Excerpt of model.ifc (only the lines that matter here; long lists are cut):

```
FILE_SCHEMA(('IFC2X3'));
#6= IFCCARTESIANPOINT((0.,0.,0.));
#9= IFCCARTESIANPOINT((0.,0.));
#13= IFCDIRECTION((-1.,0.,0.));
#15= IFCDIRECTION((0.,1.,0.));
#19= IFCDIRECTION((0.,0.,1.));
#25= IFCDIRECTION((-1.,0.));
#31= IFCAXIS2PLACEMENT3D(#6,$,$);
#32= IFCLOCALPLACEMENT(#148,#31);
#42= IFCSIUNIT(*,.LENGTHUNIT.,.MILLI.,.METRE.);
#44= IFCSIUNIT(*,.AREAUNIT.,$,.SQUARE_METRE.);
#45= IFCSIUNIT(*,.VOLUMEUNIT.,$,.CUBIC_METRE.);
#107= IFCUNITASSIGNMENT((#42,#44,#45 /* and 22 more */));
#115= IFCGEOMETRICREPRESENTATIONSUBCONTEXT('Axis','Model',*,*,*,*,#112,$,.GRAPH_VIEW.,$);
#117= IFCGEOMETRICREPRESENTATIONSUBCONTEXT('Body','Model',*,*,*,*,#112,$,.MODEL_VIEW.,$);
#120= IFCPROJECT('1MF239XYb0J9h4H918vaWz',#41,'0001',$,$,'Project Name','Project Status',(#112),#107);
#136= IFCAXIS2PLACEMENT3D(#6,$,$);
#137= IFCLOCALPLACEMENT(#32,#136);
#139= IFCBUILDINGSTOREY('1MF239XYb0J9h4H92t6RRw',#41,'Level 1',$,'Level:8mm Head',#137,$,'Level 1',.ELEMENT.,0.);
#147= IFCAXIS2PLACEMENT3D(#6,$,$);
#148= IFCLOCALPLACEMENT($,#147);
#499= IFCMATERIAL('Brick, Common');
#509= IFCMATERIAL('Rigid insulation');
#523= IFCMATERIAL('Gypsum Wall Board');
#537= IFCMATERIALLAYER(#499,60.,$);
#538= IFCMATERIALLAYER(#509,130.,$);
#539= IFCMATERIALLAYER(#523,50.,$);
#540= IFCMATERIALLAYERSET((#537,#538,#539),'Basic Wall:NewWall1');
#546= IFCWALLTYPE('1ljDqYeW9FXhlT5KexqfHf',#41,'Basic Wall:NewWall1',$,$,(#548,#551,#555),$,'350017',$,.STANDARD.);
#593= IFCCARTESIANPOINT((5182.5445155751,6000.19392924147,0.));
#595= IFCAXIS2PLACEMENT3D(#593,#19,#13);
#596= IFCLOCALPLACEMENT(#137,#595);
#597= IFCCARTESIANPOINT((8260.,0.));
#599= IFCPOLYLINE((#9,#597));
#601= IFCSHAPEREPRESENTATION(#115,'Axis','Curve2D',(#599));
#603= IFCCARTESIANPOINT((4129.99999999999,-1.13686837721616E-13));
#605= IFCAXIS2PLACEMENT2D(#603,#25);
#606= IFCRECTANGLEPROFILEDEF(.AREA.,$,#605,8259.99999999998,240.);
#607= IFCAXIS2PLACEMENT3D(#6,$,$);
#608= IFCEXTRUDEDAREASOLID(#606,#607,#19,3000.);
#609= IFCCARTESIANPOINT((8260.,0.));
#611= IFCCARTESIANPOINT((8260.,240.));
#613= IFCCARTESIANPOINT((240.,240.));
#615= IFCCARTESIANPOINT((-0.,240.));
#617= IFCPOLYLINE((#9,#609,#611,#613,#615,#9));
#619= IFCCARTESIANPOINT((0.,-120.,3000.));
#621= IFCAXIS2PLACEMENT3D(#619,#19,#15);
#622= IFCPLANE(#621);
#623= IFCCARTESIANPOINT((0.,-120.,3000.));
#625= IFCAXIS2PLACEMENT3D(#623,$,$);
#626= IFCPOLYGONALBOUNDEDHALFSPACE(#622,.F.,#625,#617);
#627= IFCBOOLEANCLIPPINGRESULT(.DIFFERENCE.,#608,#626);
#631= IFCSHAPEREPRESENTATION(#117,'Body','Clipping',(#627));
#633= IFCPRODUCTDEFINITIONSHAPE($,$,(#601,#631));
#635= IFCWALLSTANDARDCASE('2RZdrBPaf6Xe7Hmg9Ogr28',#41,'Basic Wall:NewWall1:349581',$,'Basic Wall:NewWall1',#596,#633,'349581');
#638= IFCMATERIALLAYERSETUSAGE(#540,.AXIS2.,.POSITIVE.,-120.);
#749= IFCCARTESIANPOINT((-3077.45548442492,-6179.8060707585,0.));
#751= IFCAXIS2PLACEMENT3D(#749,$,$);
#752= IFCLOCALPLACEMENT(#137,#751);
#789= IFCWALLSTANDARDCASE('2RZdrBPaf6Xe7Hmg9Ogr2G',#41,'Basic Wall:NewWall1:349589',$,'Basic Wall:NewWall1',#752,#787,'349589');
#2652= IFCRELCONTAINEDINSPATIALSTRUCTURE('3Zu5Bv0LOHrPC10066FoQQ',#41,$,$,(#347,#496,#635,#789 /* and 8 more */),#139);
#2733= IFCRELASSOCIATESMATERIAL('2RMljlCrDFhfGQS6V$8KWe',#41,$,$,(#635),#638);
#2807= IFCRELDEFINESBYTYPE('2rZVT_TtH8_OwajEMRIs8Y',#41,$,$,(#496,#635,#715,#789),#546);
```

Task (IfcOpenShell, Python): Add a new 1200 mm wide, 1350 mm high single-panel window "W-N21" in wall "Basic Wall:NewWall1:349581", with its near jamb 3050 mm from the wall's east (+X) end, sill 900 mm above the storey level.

```python
import numpy as np
import ifcopenshell
import ifcopenshell.api.feature
import ifcopenshell.api.geometry
import ifcopenshell.api.root
import ifcopenshell.api.spatial
import ifcopenshell.api.type
import ifcopenshell.geom
import ifcopenshell.util.element
import ifcopenshell.util.placement
import ifcopenshell.util.representation
import ifcopenshell.util.shape
import ifcopenshell.util.unit

model = ifcopenshell.open("model.ifc")
unit_scale = ifcopenshell.util.unit.calculate_unit_scale(model)
settings = ifcopenshell.geom.settings()


def volume(element):
    """Net volume in cubic metres, openings subtracted."""
    shape = ifcopenshell.geom.create_shape(settings, element)
    return ifcopenshell.util.shape.get_volume(shape.geometry)


wall = model.by_guid("2RZdrBPaf6Xe7Hmg9Ogr28")
storey = ifcopenshell.util.element.get_container(wall, ifc_class="IfcBuildingStorey")
context = ifcopenshell.util.representation.get_context(model, "Model", "Body", "MODEL_VIEW")
before = volume(wall)

width, height, from_end, sill = 1.2, 1.35, 3.05, 0.9  # metres

# The wall runs along its own X axis, and the end named is its -X end.
wall_shape = ifcopenshell.geom.create_shape(settings, wall)
x, y, z = ifcopenshell.util.shape.get_vertices(wall_shape.geometry).T
start = x.min() + from_end
face, thickness = float(y.min()), float(y.max() - y.min())
wall_matrix = ifcopenshell.util.placement.get_local_placement(wall.ObjectPlacement)
level = ifcopenshell.util.placement.get_local_placement(storey.ObjectPlacement)[2, 3]


def in_wall(x, y):
    """Placement at x, y metres in the wall's axes, at sill height."""
    matrix = wall_matrix.copy()
    matrix[:, 3] = wall_matrix @ np.array([x / unit_scale, y / unit_scale, 0.0, 1.0])
    matrix[2, 3] = level + sill / unit_scale
    return matrix


# Opening: a box that overshoots both wall faces by 50 mm.
opening = ifcopenshell.api.root.create_entity(model, ifc_class="IfcOpeningElement")
box = ifcopenshell.api.geometry.add_wall_representation(
    model, context=context, length=width, height=height, thickness=thickness + 0.1
)
ifcopenshell.api.geometry.assign_representation(model, product=opening, representation=box)
ifcopenshell.api.geometry.edit_object_placement(model, product=opening, matrix=in_wall(start, face - 0.05), is_si=False)
ifcopenshell.api.feature.add_feature(model, feature=opening, element=wall)

window = ifcopenshell.api.root.create_entity(model, ifc_class="IfcWindow", name="W-N21")
window.OverallWidth, window.OverallHeight = width / unit_scale, height / unit_scale
body = ifcopenshell.api.geometry.add_window_representation(
    model,
    context=context,
    overall_width=window.OverallWidth,
    overall_height=window.OverallHeight,
    partition_type="SINGLE_PANEL",
)
ifcopenshell.api.geometry.assign_representation(model, product=window, representation=body)
ifcopenshell.api.spatial.assign_container(model, products=[window], relating_structure=storey)
fills = ifcopenshell.api.feature.add_filling(model, opening=opening, element=window)
fills.OwnerHistory = window.OwnerHistory  # required in IFC2X3

# IFC2X3 keeps the operation on the window style.
style = ifcopenshell.api.root.create_entity(model, ifc_class="IfcWindowStyle", name="W-N21")
style.OperationType, style.ConstructionType = "SINGLE_PANEL", "NOTDEFINED"
style.ParameterTakesPrecedence = style.Sizeable = False
ifcopenshell.api.type.assign_type(model, related_objects=[window], relating_type=style)

# Centre the window in the wall's thickness.
ifcopenshell.api.geometry.edit_object_placement(model, product=window, matrix=in_wall(start, face), is_si=False)
window_shape = ifcopenshell.geom.create_shape(settings, window)
depth = ifcopenshell.util.shape.get_vertices(window_shape.geometry)[:, 1]
offset = face + thickness / 2 - (depth.min() + depth.max()) / 2
ifcopenshell.api.geometry.edit_object_placement(model, product=window, matrix=in_wall(start, offset), is_si=False)

after = volume(wall)

print(f"wall volume {before:.3f} -> {after:.3f} m3")

model.write("model_edited.ifc")
```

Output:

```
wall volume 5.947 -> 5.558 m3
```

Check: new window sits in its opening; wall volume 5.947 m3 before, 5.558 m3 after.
